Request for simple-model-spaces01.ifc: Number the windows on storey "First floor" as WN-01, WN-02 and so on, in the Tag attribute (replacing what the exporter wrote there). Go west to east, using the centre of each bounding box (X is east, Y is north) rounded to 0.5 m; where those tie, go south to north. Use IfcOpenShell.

First a look at what the model holds.

```python
import ifcopenshell
import ifcopenshell.util.element
import ifcopenshell.util.placement

model = ifcopenshell.open("simple-model-spaces01.ifc")
print(model.schema)
storey = next(s for s in model.by_type("IfcBuildingStorey") if s.Name == "First floor")
windows = [e for e in ifcopenshell.util.element.get_decomposition(storey) if e.is_a("IfcWindow")]
for e in sorted(windows, key=lambda e: e.id()):
    origin = ifcopenshell.util.placement.get_local_placement(e.ObjectPlacement)[:3, 3]
    print(e.id(), e.Tag, e.Name, origin.round(2) + 0.0, sep=" | ")
```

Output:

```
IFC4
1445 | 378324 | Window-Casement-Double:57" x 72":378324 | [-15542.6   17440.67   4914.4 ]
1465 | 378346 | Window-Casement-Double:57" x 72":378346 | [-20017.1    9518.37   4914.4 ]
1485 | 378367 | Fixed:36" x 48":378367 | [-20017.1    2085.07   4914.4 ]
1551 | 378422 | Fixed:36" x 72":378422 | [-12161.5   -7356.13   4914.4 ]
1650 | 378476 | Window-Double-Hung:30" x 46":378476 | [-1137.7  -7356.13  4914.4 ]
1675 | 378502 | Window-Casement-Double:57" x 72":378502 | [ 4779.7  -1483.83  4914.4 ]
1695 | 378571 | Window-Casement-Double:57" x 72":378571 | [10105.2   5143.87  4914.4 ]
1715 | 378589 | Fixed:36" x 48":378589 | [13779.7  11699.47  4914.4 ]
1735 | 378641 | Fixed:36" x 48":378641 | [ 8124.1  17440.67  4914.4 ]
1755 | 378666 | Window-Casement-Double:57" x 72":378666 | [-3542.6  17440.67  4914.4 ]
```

```python
import ifcopenshell
import ifcopenshell.geom
import ifcopenshell.util.element
import ifcopenshell.util.shape

model = ifcopenshell.open("simple-model-spaces01.ifc")
settings = ifcopenshell.geom.settings()
settings.set("use-world-coords", True)


def centre(element):
    shape = ifcopenshell.geom.create_shape(settings, element)
    return ifcopenshell.util.shape.get_bbox_centroid(shape.geometry)


storey = next(s for s in model.by_type("IfcBuildingStorey") if s.Name == "First floor")
windows = [e for e in ifcopenshell.util.element.get_decomposition(storey) if e.is_a("IfcWindow")]

# Insertion points can sit at a corner or the storey origin, so sort by the geometry (in metres).
centres = {e: centre(e) for e in windows}
windows.sort(key=lambda e: (round(centres[e][0] / 0.5), centres[e][1]))

for i, e in enumerate(windows, start=1):
    number = f"WN-{i:02d}"
    e.Tag = number
    print(e.id(), number)

model.write("simple-model-spaces01_edited.ifc")
```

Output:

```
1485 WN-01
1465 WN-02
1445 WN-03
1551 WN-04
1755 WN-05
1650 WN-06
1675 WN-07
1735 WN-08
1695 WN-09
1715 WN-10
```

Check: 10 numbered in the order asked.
